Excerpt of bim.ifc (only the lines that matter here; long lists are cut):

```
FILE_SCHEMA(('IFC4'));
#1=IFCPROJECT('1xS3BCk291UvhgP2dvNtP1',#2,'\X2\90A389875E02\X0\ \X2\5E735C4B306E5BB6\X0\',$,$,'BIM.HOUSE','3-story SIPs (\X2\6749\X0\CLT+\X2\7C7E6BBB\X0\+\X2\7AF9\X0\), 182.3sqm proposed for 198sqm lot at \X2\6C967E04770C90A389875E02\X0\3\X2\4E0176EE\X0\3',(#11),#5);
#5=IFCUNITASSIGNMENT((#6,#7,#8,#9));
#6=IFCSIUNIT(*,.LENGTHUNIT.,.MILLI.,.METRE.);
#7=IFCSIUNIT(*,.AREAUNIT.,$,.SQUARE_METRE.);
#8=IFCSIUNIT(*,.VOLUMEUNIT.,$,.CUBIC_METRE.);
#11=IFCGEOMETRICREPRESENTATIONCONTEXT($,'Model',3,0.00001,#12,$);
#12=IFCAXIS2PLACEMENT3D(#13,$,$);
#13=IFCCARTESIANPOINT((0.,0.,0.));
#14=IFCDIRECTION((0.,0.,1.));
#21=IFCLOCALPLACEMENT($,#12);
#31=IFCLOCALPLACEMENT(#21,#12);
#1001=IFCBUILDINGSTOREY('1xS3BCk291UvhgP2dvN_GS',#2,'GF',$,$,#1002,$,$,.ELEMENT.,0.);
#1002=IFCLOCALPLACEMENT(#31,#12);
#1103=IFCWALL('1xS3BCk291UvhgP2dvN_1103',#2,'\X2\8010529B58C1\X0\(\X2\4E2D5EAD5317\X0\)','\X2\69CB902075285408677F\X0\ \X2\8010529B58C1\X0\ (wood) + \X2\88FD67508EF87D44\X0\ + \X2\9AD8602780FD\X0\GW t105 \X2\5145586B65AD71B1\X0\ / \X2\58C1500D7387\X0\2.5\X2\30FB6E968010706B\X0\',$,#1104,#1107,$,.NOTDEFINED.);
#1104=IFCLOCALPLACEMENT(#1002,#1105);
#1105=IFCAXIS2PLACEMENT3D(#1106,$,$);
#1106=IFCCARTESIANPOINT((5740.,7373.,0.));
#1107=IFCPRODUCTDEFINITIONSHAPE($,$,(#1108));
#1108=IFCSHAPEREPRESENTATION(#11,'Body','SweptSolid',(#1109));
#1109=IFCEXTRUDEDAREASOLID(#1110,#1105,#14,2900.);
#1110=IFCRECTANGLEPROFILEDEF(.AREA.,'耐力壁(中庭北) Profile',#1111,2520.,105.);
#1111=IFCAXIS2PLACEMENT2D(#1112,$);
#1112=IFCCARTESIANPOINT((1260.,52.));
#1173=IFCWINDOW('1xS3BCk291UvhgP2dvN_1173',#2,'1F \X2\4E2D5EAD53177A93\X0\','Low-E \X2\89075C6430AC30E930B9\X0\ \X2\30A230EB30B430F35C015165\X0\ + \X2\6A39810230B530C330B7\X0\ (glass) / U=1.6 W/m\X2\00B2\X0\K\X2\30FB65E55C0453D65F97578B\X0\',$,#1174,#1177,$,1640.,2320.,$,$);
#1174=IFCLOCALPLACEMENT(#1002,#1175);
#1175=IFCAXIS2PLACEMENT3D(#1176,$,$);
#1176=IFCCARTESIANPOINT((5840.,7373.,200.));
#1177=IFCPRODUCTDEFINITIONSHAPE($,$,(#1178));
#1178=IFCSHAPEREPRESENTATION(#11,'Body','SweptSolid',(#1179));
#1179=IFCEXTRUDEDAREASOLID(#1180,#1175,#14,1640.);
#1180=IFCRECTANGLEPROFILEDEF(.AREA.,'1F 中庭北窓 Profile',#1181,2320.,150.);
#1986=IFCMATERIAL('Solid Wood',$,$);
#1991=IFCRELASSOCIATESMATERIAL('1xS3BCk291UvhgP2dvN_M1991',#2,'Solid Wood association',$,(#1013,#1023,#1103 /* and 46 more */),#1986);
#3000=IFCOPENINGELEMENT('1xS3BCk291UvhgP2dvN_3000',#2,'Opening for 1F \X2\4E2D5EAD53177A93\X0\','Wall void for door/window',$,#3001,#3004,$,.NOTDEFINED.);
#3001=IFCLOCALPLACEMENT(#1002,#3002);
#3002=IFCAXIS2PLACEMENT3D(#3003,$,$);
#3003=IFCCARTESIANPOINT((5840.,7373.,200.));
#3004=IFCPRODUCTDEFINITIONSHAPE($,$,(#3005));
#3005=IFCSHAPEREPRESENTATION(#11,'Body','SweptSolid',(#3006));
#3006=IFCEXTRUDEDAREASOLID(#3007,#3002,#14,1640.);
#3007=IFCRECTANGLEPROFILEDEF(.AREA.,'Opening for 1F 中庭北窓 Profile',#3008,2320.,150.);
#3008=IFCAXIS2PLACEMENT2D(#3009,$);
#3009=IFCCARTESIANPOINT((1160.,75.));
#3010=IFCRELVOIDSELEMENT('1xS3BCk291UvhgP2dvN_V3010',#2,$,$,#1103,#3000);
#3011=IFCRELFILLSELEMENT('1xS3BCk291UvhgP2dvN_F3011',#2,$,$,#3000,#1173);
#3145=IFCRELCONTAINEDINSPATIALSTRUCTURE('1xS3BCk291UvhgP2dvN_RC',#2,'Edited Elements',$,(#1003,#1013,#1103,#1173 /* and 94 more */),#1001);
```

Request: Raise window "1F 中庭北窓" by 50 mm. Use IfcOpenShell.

```python
import numpy as np
import ifcopenshell
import ifcopenshell.api.geometry
import ifcopenshell.util.placement
import ifcopenshell.util.unit

model = ifcopenshell.open("bim.ifc")
unit_scale = ifcopenshell.util.unit.calculate_unit_scale(model)

window = model.by_guid("1xS3BCk291UvhgP2dvN_1173")
opening = window.FillsVoids[0].RelatingOpeningElement
dz = 0.05 / unit_scale

shift = np.array([0.0, 0.0, dz])
# The window is not placed relative to its opening, so move both.
for product in (opening, window):
    matrix = ifcopenshell.util.placement.get_local_placement(product.ObjectPlacement)
    matrix[:3, 3] += shift
    ifcopenshell.api.geometry.edit_object_placement(model, product=product, matrix=matrix, is_si=False)

print(f"moved by {dz * unit_scale:+.3f} m")

model.write("bim-out.ifc")
```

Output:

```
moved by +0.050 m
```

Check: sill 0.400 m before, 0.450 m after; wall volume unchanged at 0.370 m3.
